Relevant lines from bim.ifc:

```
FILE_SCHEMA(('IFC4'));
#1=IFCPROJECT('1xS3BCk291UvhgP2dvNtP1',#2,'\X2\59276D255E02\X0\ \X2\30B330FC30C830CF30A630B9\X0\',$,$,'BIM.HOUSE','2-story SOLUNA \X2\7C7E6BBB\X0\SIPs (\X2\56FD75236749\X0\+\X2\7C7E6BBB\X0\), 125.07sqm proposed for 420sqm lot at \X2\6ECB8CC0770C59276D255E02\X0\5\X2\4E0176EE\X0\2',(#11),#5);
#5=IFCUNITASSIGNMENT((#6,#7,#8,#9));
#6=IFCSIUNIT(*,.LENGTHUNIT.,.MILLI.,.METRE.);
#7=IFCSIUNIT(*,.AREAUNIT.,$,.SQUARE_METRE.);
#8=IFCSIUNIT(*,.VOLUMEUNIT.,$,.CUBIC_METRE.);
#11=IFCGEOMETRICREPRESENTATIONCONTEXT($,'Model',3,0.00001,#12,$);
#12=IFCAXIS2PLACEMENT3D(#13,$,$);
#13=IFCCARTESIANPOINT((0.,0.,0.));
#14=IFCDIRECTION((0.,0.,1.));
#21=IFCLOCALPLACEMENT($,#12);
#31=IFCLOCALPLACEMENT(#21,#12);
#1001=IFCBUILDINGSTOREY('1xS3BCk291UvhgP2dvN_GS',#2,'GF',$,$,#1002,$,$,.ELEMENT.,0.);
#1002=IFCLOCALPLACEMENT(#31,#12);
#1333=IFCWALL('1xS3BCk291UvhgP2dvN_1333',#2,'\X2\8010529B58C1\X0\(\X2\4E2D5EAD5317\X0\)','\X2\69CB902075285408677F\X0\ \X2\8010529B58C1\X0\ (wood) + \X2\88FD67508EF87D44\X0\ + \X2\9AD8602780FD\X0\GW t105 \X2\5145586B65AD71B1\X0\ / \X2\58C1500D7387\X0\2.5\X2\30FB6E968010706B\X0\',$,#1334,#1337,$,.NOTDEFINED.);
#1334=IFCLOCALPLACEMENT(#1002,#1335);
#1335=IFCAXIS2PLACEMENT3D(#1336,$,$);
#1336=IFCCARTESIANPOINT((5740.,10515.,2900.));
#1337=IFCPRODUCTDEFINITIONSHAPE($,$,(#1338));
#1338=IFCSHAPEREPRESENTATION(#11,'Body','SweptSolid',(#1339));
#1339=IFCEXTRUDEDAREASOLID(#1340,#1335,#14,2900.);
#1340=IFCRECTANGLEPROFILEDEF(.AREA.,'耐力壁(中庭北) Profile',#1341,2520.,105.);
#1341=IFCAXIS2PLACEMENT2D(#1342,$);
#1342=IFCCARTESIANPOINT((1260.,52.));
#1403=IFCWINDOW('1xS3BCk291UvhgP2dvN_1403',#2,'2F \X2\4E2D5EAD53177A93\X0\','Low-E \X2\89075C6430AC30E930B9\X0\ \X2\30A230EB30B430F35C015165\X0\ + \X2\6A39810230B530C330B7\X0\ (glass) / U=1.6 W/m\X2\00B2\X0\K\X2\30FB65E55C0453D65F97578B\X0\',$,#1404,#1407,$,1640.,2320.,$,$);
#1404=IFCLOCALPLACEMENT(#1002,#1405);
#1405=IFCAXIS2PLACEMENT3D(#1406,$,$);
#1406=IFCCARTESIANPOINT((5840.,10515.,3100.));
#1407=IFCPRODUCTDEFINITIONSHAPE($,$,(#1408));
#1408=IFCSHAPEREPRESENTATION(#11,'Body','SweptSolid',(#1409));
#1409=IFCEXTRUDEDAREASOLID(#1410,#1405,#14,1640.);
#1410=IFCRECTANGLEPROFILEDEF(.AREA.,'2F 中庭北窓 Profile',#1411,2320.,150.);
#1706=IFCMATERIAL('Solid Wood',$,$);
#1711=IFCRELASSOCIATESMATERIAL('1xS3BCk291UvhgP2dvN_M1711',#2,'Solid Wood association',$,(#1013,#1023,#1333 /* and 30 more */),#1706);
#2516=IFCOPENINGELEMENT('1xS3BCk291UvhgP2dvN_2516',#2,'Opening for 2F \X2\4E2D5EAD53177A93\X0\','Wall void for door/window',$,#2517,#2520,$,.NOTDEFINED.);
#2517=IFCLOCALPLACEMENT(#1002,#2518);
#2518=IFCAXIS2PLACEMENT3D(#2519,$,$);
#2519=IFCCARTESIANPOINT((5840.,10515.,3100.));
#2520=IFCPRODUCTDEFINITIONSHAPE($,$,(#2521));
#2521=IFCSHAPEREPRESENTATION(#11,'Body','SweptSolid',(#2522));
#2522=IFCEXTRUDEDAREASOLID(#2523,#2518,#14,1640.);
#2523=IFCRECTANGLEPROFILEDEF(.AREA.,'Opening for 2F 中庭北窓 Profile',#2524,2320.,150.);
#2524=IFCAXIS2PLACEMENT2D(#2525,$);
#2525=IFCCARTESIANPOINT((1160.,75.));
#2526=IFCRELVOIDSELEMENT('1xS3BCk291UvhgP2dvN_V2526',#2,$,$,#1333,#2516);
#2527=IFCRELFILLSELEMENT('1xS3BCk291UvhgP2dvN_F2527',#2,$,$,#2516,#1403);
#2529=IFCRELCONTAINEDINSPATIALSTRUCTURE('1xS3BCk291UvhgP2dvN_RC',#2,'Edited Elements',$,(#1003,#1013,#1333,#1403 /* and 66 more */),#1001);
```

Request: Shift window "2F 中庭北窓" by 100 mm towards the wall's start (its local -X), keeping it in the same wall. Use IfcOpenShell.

```python
import ifcopenshell
import ifcopenshell.api.geometry
import ifcopenshell.util.placement

model = ifcopenshell.open("bim.ifc")

window = model.by_id(1403)
opening = window.FillsVoids[0].RelatingOpeningElement
wall = opening.VoidsElements[0].RelatingBuildingElement

wall_matrix = ifcopenshell.util.placement.get_local_placement(wall.ObjectPlacement)
shift = wall_matrix[:3, 0] * -100.0
before = ifcopenshell.util.placement.get_local_placement(window.ObjectPlacement)[:3, 3].copy()

# The window is not placed relative to its opening, so move both.
for product in (opening, window):
    matrix = ifcopenshell.util.placement.get_local_placement(product.ObjectPlacement)
    matrix[:3, 3] += shift
    ifcopenshell.api.geometry.edit_object_placement(model, product=product, matrix=matrix, is_si=False)

after = ifcopenshell.util.placement.get_local_placement(window.ObjectPlacement)[:3, 3]
print("window moved by", (after - before).round(3) + 0.0)

model.write("bim_edited.ifc")
```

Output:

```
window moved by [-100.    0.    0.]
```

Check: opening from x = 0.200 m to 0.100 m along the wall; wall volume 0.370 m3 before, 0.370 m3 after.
